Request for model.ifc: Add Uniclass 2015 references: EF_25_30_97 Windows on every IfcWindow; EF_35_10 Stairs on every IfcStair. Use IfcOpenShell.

First a look at what the model holds.

```python
import ifcopenshell

model = ifcopenshell.open("model.ifc")
print(model.schema)
print("classifications:", [c.Name for c in model.by_type("IfcClassification")])
for ifc_class in ("IfcDoor", "IfcRoof", "IfcStair", "IfcWall", "IfcWindow"):
    print(ifc_class, len(model.by_type(ifc_class)))
```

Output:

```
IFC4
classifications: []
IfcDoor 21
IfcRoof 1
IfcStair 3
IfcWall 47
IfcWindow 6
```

```python
import ifcopenshell
import ifcopenshell.api.classification

model = ifcopenshell.open("model.ifc")

system = ifcopenshell.api.classification.add_classification(model, classification="Uniclass 2015")

codes = {
    "IfcWindow": ("EF_25_30_97", "Windows"),
    "IfcStair": ("EF_35_10", "Stairs"),
}
for ifc_class, (code, name) in codes.items():
    products = model.by_type(ifc_class)
    ifcopenshell.api.classification.add_reference(
        model, products=products, classification=system, identification=code, name=name
    )
    print(code, len(products))

model.write("model_rev.ifc")
```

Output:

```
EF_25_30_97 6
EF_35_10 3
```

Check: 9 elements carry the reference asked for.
